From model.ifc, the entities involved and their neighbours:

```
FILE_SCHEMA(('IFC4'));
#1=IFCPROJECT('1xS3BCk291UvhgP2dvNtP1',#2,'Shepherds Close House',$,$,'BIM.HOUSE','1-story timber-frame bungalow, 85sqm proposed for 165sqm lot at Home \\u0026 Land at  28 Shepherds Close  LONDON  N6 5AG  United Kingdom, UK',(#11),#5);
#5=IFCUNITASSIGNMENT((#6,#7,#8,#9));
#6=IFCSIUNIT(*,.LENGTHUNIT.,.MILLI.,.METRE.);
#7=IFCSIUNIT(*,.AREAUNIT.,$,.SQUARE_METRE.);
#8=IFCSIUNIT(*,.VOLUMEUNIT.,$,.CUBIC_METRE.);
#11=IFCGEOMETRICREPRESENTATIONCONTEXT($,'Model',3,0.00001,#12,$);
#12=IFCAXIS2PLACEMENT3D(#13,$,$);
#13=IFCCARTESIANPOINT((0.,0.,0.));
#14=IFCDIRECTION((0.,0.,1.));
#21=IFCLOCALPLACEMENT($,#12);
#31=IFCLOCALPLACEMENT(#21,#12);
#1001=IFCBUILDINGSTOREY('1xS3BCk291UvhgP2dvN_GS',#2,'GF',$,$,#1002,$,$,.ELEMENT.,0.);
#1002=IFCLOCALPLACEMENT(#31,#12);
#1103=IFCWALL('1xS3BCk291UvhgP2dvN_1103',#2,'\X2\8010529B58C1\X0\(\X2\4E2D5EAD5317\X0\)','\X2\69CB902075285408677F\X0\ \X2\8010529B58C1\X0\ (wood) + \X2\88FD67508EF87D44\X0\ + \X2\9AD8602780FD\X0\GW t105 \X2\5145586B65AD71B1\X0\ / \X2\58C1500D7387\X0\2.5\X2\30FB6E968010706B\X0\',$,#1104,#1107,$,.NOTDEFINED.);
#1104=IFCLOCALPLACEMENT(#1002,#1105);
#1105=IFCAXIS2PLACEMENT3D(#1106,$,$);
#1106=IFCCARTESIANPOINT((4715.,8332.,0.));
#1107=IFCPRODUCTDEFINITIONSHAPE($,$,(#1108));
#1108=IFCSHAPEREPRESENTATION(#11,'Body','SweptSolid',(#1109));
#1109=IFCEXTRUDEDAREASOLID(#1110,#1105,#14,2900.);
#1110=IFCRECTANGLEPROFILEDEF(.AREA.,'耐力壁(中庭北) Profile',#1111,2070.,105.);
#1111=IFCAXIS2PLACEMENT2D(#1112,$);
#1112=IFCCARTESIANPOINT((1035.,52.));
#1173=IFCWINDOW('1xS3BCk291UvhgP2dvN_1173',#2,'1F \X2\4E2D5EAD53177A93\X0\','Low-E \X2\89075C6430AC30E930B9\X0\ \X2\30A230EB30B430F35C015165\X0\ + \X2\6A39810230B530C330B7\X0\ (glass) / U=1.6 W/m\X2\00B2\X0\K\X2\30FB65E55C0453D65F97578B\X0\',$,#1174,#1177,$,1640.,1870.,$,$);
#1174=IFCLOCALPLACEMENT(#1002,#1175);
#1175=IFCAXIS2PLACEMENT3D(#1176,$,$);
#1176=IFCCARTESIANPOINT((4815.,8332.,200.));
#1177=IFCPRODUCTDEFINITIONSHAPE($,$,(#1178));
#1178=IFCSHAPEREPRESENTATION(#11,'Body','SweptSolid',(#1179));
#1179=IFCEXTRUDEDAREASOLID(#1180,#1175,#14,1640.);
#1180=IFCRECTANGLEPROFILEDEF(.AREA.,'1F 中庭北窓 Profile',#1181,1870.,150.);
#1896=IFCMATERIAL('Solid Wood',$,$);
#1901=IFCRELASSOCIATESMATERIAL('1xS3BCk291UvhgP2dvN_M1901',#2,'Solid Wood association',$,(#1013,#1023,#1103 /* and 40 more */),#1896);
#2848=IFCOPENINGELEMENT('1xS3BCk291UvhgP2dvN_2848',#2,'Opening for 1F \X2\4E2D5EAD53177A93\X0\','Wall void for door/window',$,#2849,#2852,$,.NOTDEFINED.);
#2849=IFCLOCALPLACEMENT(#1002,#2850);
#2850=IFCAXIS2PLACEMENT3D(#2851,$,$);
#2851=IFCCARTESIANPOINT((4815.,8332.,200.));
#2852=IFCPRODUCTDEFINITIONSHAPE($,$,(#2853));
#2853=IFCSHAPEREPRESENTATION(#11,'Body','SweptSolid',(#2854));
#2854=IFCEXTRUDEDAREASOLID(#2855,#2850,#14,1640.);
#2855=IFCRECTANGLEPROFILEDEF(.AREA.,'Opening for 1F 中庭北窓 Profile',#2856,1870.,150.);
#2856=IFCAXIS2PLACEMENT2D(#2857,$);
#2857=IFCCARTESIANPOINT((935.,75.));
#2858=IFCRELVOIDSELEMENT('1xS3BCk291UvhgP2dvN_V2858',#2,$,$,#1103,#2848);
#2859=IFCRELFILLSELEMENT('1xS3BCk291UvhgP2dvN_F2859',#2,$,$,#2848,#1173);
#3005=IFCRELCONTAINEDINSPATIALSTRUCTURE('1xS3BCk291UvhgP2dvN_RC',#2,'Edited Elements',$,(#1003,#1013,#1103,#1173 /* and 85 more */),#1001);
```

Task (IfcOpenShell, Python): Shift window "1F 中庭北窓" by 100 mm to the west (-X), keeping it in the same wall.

```python
import ifcopenshell
import ifcopenshell.api.geometry
import ifcopenshell.util.placement
import ifcopenshell.util.unit

model = ifcopenshell.open("model.ifc")
unit_scale = ifcopenshell.util.unit.calculate_unit_scale(model)

window = model.by_guid("1xS3BCk291UvhgP2dvN_1173")
opening = window.FillsVoids[0].RelatingOpeningElement
wall = opening.VoidsElements[0].RelatingBuildingElement

wall_matrix = ifcopenshell.util.placement.get_local_placement(wall.ObjectPlacement)
shift = wall_matrix[:3, 0] * -0.1 / unit_scale
before = ifcopenshell.util.placement.get_local_placement(window.ObjectPlacement)[:3, 3].copy()

# The window is not placed relative to its opening, so move both.
for product in (opening, window):
    matrix = ifcopenshell.util.placement.get_local_placement(product.ObjectPlacement)
    matrix[:3, 3] += shift
    ifcopenshell.api.geometry.edit_object_placement(model, product=product, matrix=matrix, is_si=False)

after = ifcopenshell.util.placement.get_local_placement(window.ObjectPlacement)[:3, 3]
print("window moved by", (after - before).round(3) + 0.0)

model.write("model_rev.ifc")
```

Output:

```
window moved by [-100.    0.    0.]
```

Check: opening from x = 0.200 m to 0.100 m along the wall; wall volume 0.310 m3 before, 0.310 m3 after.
